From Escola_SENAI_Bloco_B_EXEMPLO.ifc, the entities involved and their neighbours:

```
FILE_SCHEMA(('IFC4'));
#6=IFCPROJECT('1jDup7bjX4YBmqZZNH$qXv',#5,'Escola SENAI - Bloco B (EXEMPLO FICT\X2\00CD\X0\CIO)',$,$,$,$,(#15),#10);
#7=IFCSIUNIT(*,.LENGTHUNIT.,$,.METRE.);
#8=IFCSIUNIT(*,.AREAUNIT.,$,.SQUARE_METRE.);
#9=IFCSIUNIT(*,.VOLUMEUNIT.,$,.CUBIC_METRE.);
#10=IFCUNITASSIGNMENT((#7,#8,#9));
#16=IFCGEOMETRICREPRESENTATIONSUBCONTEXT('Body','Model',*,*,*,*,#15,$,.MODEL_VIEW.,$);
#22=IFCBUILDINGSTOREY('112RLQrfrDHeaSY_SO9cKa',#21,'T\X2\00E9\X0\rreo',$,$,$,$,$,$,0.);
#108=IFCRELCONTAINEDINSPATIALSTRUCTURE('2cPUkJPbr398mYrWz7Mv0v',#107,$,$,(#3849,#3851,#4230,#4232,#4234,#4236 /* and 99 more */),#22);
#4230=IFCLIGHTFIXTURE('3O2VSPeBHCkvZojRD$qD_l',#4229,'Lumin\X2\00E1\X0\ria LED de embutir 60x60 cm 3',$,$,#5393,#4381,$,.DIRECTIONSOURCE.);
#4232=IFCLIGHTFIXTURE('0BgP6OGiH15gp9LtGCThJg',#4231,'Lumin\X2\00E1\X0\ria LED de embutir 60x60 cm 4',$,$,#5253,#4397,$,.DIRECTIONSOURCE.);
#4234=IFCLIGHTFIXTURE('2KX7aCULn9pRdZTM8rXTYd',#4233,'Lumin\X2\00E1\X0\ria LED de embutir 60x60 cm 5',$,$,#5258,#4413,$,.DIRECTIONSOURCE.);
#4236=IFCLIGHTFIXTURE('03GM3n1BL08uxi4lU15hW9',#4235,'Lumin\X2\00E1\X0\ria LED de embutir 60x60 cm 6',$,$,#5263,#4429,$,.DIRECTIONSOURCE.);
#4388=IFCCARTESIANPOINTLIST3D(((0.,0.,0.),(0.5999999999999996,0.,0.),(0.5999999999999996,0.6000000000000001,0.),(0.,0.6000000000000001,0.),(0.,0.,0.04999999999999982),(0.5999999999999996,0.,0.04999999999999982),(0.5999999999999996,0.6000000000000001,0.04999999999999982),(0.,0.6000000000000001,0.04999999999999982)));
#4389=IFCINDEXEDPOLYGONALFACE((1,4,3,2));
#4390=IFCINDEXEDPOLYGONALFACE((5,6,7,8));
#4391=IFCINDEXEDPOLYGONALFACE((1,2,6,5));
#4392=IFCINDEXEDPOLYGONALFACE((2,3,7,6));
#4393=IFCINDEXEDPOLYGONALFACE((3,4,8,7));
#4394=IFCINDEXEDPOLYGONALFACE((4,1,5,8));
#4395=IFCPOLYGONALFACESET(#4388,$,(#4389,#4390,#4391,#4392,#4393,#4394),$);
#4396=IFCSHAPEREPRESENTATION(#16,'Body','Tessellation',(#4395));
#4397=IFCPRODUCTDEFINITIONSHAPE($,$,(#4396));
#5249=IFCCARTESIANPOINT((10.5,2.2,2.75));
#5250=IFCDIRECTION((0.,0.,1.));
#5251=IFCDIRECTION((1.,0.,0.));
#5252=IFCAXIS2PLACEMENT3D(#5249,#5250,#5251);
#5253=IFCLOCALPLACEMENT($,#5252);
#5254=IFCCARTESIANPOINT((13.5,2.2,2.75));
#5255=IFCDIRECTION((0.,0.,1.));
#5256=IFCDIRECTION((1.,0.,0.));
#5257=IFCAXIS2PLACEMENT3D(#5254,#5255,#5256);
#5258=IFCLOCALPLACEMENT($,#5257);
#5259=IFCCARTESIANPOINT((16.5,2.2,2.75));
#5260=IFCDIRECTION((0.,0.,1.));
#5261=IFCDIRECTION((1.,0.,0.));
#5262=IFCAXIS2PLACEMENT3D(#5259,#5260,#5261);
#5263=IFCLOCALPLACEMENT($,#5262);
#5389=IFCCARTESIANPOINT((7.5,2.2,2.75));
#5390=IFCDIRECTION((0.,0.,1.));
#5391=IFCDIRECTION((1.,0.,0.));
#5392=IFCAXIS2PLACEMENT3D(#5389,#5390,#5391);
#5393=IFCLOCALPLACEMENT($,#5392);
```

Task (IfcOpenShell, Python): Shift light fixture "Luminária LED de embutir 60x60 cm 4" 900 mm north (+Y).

```python
import ifcopenshell
import ifcopenshell.api.geometry
import ifcopenshell.util.placement
import ifcopenshell.util.unit

model = ifcopenshell.open("Escola_SENAI_Bloco_B_EXEMPLO.ifc")
unit_scale = ifcopenshell.util.unit.calculate_unit_scale(model)

item = model.by_guid("0BgP6OGiH15gp9LtGCThJg")
matrix = ifcopenshell.util.placement.get_local_placement(item.ObjectPlacement)
matrix[1, 3] += 0.9 / unit_scale
ifcopenshell.api.geometry.edit_object_placement(model, product=item, matrix=matrix, is_si=False)

print(ifcopenshell.util.placement.get_local_placement(item.ObjectPlacement).round(3) + 0.0)

model.write("Escola_SENAI_Bloco_B_EXEMPLO_edited.ifc")
```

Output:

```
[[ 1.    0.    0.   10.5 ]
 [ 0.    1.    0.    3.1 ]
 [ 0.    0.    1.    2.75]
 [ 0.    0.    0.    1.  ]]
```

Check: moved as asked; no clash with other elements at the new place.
